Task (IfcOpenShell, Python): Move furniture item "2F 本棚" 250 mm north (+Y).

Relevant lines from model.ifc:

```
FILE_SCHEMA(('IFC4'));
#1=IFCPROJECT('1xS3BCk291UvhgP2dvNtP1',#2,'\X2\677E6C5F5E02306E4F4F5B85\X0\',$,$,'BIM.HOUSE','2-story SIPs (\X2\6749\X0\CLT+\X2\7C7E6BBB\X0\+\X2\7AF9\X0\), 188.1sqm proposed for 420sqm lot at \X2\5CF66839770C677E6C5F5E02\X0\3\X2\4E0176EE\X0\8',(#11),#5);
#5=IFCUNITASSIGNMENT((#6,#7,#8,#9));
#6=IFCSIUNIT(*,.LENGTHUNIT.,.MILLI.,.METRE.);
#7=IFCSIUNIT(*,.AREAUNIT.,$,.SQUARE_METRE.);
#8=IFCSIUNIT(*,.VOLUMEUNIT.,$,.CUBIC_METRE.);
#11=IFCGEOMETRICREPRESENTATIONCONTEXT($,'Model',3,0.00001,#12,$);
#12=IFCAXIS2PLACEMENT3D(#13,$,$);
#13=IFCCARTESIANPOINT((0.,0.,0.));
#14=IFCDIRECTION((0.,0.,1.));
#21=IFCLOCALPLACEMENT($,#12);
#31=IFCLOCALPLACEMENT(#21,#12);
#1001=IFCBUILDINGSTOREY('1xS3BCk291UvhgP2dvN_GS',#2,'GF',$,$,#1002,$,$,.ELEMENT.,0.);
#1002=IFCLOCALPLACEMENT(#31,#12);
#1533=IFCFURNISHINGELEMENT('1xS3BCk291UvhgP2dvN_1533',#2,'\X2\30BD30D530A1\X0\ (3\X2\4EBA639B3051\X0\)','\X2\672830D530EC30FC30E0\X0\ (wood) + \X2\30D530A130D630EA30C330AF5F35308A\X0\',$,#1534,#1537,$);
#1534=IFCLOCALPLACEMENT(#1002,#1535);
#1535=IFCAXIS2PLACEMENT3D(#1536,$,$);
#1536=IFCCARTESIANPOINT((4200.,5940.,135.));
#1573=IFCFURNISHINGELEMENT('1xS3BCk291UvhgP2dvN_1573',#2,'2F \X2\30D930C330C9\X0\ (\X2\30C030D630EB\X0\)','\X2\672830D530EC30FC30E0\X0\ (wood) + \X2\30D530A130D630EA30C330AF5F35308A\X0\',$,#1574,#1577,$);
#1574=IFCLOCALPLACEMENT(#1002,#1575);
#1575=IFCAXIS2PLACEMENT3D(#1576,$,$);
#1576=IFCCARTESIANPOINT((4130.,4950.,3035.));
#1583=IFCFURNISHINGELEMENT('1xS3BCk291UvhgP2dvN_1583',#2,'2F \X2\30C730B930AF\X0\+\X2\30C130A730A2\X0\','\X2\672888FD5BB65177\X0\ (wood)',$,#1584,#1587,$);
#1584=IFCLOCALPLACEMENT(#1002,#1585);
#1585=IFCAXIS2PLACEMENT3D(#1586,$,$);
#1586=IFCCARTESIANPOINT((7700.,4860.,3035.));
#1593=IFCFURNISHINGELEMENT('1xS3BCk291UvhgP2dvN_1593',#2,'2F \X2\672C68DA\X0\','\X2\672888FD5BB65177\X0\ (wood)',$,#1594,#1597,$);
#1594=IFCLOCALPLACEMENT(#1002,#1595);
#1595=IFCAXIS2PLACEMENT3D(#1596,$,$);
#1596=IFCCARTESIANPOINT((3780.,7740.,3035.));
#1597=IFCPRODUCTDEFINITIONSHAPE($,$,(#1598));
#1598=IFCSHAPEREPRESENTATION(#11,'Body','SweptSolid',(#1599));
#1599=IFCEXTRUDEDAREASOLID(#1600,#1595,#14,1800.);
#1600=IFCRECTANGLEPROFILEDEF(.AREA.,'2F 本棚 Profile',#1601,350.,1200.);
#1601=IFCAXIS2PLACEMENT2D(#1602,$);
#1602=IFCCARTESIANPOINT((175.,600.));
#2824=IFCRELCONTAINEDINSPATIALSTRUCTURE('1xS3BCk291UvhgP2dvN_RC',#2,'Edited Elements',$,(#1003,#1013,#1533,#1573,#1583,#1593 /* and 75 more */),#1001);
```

```python
import ifcopenshell
import ifcopenshell.api.geometry
import ifcopenshell.util.placement
import ifcopenshell.util.unit

model = ifcopenshell.open("model.ifc")
unit_scale = ifcopenshell.util.unit.calculate_unit_scale(model)

item = model.by_guid("1xS3BCk291UvhgP2dvN_1593")
matrix = ifcopenshell.util.placement.get_local_placement(item.ObjectPlacement)
matrix[1, 3] += 0.25 / unit_scale
ifcopenshell.api.geometry.edit_object_placement(model, product=item, matrix=matrix, is_si=False)

print(ifcopenshell.util.placement.get_local_placement(item.ObjectPlacement).round(3) + 0.0)

model.write("model_updated.ifc")
```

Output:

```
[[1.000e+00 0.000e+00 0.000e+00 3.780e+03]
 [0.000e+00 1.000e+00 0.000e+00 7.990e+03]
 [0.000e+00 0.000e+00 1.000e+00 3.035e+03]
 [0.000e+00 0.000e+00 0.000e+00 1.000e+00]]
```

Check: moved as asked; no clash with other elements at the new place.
